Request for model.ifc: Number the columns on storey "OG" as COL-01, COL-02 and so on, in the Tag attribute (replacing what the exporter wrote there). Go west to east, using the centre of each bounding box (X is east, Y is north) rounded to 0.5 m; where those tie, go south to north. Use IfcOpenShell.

First a look at what the model holds.

```python
import ifcopenshell
import ifcopenshell.util.element
import ifcopenshell.util.placement

model = ifcopenshell.open("model.ifc")
print(model.schema)
storey = next(s for s in model.by_type("IfcBuildingStorey") if s.Name == "OG")
columns = [e for e in ifcopenshell.util.element.get_decomposition(storey) if e.is_a("IfcColumn")]
for e in sorted(columns, key=lambda e: e.id()):
    origin = ifcopenshell.util.placement.get_local_placement(e.ObjectPlacement)[:3, 3]
    print(e.id(), e.Tag, e.Name, origin.round(2) + 0.0, sep=" | ")
```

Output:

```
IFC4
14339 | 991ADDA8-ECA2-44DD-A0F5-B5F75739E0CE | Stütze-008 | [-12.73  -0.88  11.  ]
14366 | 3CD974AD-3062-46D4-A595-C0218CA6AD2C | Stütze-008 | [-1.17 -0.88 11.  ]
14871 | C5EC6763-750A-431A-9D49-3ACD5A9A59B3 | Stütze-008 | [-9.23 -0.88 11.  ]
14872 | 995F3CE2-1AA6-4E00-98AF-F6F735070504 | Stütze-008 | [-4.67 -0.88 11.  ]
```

```python
import ifcopenshell
import ifcopenshell.geom
import ifcopenshell.util.element
import ifcopenshell.util.shape

model = ifcopenshell.open("model.ifc")
settings = ifcopenshell.geom.settings()
settings.set("use-world-coords", True)


def centre(element):
    shape = ifcopenshell.geom.create_shape(settings, element)
    return ifcopenshell.util.shape.get_bbox_centroid(shape.geometry)


storey = next(s for s in model.by_type("IfcBuildingStorey") if s.Name == "OG")
columns = [e for e in ifcopenshell.util.element.get_decomposition(storey) if e.is_a("IfcColumn")]

# Insertion points can sit at a corner or the storey origin, so sort by the geometry (in metres).
centres = {e: centre(e) for e in columns}
columns.sort(key=lambda e: (round(centres[e][0] / 0.5), centres[e][1]))

for i, e in enumerate(columns, start=1):
    number = f"COL-{i:02d}"
    e.Tag = number
    print(e.id(), number)

model.write("model-out.ifc")
```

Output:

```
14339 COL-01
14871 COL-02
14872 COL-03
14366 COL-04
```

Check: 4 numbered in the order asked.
